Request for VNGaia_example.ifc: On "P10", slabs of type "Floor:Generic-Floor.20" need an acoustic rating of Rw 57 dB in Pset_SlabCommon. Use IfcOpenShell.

First a look at what the model holds.

```python
import ifcopenshell
import ifcopenshell.util.element

model = ifcopenshell.open("VNGaia_example.ifc")
print(model.schema)
storey = next(s for s in model.by_type("IfcBuildingStorey") if s.Name == "P10")
slabs = [e for e in ifcopenshell.util.element.get_decomposition(storey) if e.is_a("IfcSlab")]
seen = {}
for e in slabs:
    element_type = ifcopenshell.util.element.get_type(e)
    key = (element_type.Name if element_type != e and element_type else None, ifcopenshell.util.element.get_pset(e, "Pset_SlabCommon", "AcousticRating"))
    seen[key] = seen.get(key, 0) + 1
for (name, value), count in sorted(seen.items(), key=str):
    print(count, "x", name, "|", value)
```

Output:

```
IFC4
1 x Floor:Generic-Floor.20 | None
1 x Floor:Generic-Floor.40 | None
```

```python
import ifcopenshell
import ifcopenshell.api.pset
import ifcopenshell.util.element

model = ifcopenshell.open("VNGaia_example.ifc")

storey = next(s for s in model.by_type("IfcBuildingStorey") if s.Name == "P10")
slabs = [e for e in ifcopenshell.util.element.get_decomposition(storey) if e.is_a("IfcSlab")]

count = 0
for e in slabs:
    element_type = ifcopenshell.util.element.get_type(e)
    if element_type in (None, e) or element_type.Name != "Floor:Generic-Floor.20":
        continue
    # add_pset returns the element's existing set when there is one.
    pset = ifcopenshell.api.pset.add_pset(model, product=e, name="Pset_SlabCommon")
    ifcopenshell.api.pset.edit_pset(model, pset=pset, properties={"AcousticRating": "Rw 57 dB"})
    count += 1

print(count, "slabs updated")

model.write("VNGaia_example-out.ifc")
```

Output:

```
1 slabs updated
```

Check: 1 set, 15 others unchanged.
